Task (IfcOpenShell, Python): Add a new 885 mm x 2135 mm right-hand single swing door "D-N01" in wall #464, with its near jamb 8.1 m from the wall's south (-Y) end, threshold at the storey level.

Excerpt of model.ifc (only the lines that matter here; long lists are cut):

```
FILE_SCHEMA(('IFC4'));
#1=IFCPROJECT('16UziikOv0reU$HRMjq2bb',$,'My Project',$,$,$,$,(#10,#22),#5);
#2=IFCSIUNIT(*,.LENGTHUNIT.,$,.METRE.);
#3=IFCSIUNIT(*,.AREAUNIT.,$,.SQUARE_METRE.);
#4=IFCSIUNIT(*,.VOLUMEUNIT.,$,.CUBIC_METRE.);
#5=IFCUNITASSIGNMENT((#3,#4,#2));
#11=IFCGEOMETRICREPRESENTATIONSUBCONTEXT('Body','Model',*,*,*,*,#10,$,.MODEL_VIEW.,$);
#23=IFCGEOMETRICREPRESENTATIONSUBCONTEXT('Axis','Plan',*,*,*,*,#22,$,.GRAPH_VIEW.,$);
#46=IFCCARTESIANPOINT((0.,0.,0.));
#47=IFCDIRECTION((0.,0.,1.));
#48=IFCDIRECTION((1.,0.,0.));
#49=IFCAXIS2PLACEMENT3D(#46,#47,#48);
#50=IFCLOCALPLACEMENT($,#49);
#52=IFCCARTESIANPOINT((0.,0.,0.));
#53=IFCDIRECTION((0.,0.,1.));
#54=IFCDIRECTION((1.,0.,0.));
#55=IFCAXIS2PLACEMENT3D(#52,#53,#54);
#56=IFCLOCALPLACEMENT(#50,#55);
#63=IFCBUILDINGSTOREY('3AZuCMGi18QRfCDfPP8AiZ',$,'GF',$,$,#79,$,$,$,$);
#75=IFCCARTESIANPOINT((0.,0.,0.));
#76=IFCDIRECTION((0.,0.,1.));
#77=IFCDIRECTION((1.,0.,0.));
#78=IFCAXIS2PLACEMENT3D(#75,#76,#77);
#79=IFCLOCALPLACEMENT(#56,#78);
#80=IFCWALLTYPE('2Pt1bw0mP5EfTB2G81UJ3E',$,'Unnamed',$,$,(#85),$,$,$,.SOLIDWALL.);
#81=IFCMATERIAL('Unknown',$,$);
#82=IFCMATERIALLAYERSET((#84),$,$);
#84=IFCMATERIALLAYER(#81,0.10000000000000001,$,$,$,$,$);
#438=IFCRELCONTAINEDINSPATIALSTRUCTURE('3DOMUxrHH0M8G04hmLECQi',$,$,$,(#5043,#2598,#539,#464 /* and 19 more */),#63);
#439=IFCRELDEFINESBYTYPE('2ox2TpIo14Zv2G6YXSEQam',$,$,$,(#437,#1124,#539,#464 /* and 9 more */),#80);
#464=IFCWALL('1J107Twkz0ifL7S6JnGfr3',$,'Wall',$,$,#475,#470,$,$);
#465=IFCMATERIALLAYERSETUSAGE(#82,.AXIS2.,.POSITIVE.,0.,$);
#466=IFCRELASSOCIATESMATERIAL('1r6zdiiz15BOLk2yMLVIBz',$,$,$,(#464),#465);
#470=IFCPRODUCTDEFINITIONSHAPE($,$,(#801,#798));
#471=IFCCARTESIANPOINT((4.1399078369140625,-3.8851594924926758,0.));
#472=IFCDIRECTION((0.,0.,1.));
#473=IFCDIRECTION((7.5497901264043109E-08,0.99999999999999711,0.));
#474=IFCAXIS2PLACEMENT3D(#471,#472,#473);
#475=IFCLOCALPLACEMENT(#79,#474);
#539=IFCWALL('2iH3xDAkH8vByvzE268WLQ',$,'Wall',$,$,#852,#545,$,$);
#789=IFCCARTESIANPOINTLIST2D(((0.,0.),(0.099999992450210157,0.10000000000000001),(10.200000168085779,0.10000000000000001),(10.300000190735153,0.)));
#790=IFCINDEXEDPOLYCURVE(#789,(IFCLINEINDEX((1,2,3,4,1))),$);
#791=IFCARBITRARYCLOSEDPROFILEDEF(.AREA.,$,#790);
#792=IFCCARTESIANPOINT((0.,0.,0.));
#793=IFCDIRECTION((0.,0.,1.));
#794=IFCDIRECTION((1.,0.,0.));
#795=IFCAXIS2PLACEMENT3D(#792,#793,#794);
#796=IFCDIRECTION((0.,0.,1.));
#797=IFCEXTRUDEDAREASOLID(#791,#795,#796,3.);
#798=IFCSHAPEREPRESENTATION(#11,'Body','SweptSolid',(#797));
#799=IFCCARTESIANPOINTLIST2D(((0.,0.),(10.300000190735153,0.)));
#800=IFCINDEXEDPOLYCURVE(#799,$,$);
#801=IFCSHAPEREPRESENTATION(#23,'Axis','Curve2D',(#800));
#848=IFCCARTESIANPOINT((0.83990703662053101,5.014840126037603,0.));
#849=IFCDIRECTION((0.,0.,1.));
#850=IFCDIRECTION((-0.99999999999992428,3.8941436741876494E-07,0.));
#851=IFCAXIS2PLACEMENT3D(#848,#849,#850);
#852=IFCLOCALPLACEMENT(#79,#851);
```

```python
import numpy as np
import ifcopenshell
import ifcopenshell.api.feature
import ifcopenshell.api.geometry
import ifcopenshell.api.root
import ifcopenshell.api.spatial
import ifcopenshell.geom
import ifcopenshell.util.element
import ifcopenshell.util.placement
import ifcopenshell.util.representation
import ifcopenshell.util.shape
import ifcopenshell.util.unit

model = ifcopenshell.open("model.ifc")
unit_scale = ifcopenshell.util.unit.calculate_unit_scale(model)
settings = ifcopenshell.geom.settings()


def volume(element):
    """Net volume in cubic metres, openings subtracted."""
    shape = ifcopenshell.geom.create_shape(settings, element)
    return ifcopenshell.util.shape.get_volume(shape.geometry)


wall = model.by_guid("1J107Twkz0ifL7S6JnGfr3")
storey = ifcopenshell.util.element.get_container(wall, ifc_class="IfcBuildingStorey")
context = ifcopenshell.util.representation.get_context(model, "Model", "Body", "MODEL_VIEW")
before = volume(wall)

width, height, from_end, sill = 0.885, 2.135, 8.1, 0.0  # metres

# The wall runs along its own X axis, and the end named is its -X end.
wall_shape = ifcopenshell.geom.create_shape(settings, wall)
x, y, z = ifcopenshell.util.shape.get_vertices(wall_shape.geometry).T
start = x.min() + from_end
face, thickness = float(y.min()), float(y.max() - y.min())
wall_matrix = ifcopenshell.util.placement.get_local_placement(wall.ObjectPlacement)
level = ifcopenshell.util.placement.get_local_placement(storey.ObjectPlacement)[2, 3]


def in_wall(x, y):
    """Placement at x, y metres in the wall's axes, at sill height."""
    matrix = wall_matrix.copy()
    matrix[:, 3] = wall_matrix @ np.array([x / unit_scale, y / unit_scale, 0.0, 1.0])
    matrix[2, 3] = level + sill / unit_scale
    return matrix


# Opening: a box that overshoots both wall faces by 50 mm.
opening = ifcopenshell.api.root.create_entity(model, ifc_class="IfcOpeningElement", predefined_type="OPENING")
box = ifcopenshell.api.geometry.add_wall_representation(
    model, context=context, length=width, height=height, thickness=thickness + 0.1
)
ifcopenshell.api.geometry.assign_representation(model, product=opening, representation=box)
ifcopenshell.api.geometry.edit_object_placement(model, product=opening, matrix=in_wall(start, face - 0.05), is_si=False)
ifcopenshell.api.feature.add_feature(model, feature=opening, element=wall)

door = ifcopenshell.api.root.create_entity(model, ifc_class="IfcDoor", name="D-N01", predefined_type="DOOR")
door.OverallWidth, door.OverallHeight = width / unit_scale, height / unit_scale
door.OperationType = "SINGLE_SWING_RIGHT"
body = ifcopenshell.api.geometry.add_door_representation(
    model,
    context=context,
    overall_width=door.OverallWidth,
    overall_height=door.OverallHeight,
    operation_type="SINGLE_SWING_RIGHT",
    lining_properties={"LiningDepth": thickness / unit_scale, "ThresholdDepth": thickness / unit_scale},
)
ifcopenshell.api.geometry.assign_representation(model, product=door, representation=body)
ifcopenshell.api.spatial.assign_container(model, products=[door], relating_structure=storey)
ifcopenshell.api.feature.add_filling(model, opening=opening, element=door)

# The lining spans the wall, so the door starts at the wall face.
ifcopenshell.api.geometry.edit_object_placement(model, product=door, matrix=in_wall(start, face), is_si=False)

after = volume(wall)

print(f"wall volume {before:.3f} -> {after:.3f} m3")

model.write("model_v2.ifc")
```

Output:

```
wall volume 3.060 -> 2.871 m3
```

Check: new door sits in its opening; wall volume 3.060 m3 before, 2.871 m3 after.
